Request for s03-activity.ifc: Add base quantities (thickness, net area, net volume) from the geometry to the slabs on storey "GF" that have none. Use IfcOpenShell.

First a look at what the model holds.

```python
import ifcopenshell
import ifcopenshell.util.element
import ifcopenshell.util.unit

model = ifcopenshell.open("s03-activity.ifc")
print(model.schema)
for unit_type in ("LENGTHUNIT", "AREAUNIT", "VOLUMEUNIT"):
    print(unit_type, ifcopenshell.util.unit.calculate_unit_scale(model, unit_type))
storey = next(s for s in model.by_type("IfcBuildingStorey") if s.Name == "GF")
slabs = [e for e in ifcopenshell.util.element.get_decomposition(storey) if e.is_a("IfcSlab")]
for e in sorted(slabs, key=lambda e: e.id()):
    print(e.id(), e.is_a(), e.Name, list(ifcopenshell.util.element.get_psets(e, qtos_only=True)), sep=" | ")
```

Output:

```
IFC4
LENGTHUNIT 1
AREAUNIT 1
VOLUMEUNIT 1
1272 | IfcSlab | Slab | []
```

```python
import ifcopenshell
import ifcopenshell.api.pset
import ifcopenshell.geom
import ifcopenshell.util.element
import ifcopenshell.util.shape
import ifcopenshell.util.unit

model = ifcopenshell.open("s03-activity.ifc")
unit_scale = ifcopenshell.util.unit.calculate_unit_scale(model)
area_scale = ifcopenshell.util.unit.calculate_unit_scale(model, "AREAUNIT")
volume_scale = ifcopenshell.util.unit.calculate_unit_scale(model, "VOLUMEUNIT")
settings = ifcopenshell.geom.settings()

storey = next(s for s in model.by_type("IfcBuildingStorey") if s.Name == "GF")
slabs = [e for e in ifcopenshell.util.element.get_decomposition(storey) if e.is_a("IfcSlab")]

for e in sorted(slabs, key=lambda e: e.id()):
    if ifcopenshell.util.element.get_psets(e, qtos_only=True, should_inherit=False):
        continue
    # Geometry comes back in metres, in the element's own axes.
    shape = ifcopenshell.geom.create_shape(settings, e)
    values = {
        "Width": ifcopenshell.util.shape.get_z(shape.geometry) / unit_scale,
        "NetArea": ifcopenshell.util.shape.get_footprint_area(shape.geometry) / area_scale,
        "NetVolume": ifcopenshell.util.shape.get_volume(shape.geometry) / volume_scale,
    }
    qto = ifcopenshell.api.pset.add_qto(model, product=e, name="Qto_SlabBaseQuantities")
    ifcopenshell.api.pset.edit_qto(model, qto=qto, properties=values)
    print(e.id(), {k: round(v, 3) for k, v in values.items()})

model.write("s03-activity_updated.ifc")
```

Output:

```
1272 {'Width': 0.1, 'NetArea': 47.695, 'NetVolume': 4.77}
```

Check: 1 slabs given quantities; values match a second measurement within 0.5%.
